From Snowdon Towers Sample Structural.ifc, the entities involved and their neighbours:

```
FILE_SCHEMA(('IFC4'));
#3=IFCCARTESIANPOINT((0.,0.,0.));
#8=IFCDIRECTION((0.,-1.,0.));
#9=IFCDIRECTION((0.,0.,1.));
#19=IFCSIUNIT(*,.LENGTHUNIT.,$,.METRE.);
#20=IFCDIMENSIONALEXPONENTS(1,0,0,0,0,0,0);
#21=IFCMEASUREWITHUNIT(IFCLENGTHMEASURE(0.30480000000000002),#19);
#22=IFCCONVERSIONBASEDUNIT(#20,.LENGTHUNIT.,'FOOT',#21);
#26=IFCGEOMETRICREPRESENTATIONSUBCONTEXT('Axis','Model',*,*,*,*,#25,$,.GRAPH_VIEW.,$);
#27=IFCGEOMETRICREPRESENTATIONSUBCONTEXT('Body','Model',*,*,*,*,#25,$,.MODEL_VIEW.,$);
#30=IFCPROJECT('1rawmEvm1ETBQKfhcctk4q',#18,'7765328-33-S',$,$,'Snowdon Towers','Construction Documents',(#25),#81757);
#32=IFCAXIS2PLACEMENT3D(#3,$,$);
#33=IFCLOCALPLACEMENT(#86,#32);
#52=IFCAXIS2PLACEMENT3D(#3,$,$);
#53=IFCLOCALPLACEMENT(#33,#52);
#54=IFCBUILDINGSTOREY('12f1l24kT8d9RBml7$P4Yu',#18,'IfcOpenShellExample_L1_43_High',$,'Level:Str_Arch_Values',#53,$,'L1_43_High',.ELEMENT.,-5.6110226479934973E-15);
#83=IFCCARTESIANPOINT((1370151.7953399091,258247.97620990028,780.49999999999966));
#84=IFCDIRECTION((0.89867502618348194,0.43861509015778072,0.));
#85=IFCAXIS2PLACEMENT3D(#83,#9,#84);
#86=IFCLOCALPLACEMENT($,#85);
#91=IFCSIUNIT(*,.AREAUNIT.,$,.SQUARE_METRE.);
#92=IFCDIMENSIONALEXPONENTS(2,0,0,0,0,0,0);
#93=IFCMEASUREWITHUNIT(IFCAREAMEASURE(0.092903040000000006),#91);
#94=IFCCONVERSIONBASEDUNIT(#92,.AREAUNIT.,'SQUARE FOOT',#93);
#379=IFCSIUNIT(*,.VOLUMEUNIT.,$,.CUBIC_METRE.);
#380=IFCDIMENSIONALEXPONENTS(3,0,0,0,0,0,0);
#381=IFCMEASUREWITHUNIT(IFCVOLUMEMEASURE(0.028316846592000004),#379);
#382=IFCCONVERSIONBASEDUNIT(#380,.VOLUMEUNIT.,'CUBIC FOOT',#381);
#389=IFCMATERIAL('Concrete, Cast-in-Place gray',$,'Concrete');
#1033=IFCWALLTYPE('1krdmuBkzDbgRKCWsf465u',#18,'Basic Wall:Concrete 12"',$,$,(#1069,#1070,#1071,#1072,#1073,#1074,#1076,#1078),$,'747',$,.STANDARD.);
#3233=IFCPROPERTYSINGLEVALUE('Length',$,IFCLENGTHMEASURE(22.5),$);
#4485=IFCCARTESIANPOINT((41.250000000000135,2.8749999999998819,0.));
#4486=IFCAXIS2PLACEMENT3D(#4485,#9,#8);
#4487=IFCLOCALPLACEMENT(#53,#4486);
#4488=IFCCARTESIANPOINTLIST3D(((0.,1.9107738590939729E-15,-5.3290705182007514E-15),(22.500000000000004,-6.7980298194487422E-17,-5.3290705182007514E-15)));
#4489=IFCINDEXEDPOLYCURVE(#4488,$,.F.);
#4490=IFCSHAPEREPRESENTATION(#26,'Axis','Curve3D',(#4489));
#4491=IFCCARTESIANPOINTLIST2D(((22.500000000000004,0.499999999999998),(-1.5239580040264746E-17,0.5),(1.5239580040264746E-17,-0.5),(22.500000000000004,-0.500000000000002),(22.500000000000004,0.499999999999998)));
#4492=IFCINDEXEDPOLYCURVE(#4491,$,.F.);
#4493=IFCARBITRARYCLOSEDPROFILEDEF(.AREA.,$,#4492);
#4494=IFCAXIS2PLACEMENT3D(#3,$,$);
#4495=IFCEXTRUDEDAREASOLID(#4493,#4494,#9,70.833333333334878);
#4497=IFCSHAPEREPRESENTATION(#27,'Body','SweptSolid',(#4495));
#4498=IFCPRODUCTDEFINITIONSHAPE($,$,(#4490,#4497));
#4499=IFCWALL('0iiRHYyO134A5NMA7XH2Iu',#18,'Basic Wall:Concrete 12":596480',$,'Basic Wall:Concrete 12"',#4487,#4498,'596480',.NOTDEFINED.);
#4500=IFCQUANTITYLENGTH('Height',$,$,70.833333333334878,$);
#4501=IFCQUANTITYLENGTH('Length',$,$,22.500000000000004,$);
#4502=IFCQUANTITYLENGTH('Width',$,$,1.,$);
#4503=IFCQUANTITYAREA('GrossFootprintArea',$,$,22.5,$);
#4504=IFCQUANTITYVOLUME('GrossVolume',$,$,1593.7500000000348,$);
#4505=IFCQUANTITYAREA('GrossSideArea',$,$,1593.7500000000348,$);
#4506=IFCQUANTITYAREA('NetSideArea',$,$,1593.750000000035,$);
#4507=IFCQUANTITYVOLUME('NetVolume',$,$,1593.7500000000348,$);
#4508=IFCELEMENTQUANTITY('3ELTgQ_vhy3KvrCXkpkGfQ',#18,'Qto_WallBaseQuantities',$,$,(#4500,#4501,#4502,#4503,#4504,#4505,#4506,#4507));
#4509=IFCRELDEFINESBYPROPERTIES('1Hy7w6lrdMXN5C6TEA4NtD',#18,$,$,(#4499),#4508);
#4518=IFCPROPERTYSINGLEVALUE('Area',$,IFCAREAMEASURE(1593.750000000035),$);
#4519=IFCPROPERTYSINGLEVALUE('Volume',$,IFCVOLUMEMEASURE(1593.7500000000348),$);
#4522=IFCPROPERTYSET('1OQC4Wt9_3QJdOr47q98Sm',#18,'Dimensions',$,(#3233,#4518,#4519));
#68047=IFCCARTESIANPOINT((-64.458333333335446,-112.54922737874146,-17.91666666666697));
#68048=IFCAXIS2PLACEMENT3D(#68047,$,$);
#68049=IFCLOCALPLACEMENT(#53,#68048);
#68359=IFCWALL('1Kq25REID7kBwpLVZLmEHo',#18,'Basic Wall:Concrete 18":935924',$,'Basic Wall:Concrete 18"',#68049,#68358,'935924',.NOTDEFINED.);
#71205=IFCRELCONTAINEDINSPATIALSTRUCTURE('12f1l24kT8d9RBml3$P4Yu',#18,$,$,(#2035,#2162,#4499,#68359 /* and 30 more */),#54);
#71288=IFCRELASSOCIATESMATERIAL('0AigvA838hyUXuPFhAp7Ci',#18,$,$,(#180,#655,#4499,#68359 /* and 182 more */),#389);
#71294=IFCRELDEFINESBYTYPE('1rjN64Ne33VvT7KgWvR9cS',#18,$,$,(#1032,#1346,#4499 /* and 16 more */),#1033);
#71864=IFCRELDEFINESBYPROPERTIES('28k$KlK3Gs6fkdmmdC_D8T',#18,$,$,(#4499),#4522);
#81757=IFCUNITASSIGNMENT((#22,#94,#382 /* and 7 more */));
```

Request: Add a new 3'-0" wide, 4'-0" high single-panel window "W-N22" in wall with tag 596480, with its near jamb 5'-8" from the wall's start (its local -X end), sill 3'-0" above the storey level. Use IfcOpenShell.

```python
import numpy as np
import ifcopenshell
import ifcopenshell.api.feature
import ifcopenshell.api.geometry
import ifcopenshell.api.pset
import ifcopenshell.api.root
import ifcopenshell.api.spatial
import ifcopenshell.geom
import ifcopenshell.util.element
import ifcopenshell.util.placement
import ifcopenshell.util.representation
import ifcopenshell.util.shape
import ifcopenshell.util.unit

model = ifcopenshell.open("Snowdon Towers Sample Structural.ifc")
unit_scale = ifcopenshell.util.unit.calculate_unit_scale(model)
area_scale = ifcopenshell.util.unit.calculate_unit_scale(model, "AREAUNIT")
volume_scale = ifcopenshell.util.unit.calculate_unit_scale(model, "VOLUMEUNIT")
settings = ifcopenshell.geom.settings()


def volume(element):
    """Net volume in cubic metres, openings subtracted."""
    shape = ifcopenshell.geom.create_shape(settings, element)
    return ifcopenshell.util.shape.get_volume(shape.geometry)


wall = model.by_guid("0iiRHYyO134A5NMA7XH2Iu")
storey = ifcopenshell.util.element.get_container(wall, ifc_class="IfcBuildingStorey")
context = ifcopenshell.util.representation.get_context(model, "Model", "Body", "MODEL_VIEW")
before = volume(wall)

width, height, from_end, sill = 0.9144, 1.2192, 1.7272, 0.9144  # metres

# The wall runs along its own X axis, and the end named is its -X end.
wall_shape = ifcopenshell.geom.create_shape(settings, wall)
x, y, z = ifcopenshell.util.shape.get_vertices(wall_shape.geometry).T
start = x.min() + from_end
face, thickness = float(y.min()), float(y.max() - y.min())
wall_matrix = ifcopenshell.util.placement.get_local_placement(wall.ObjectPlacement)
level = ifcopenshell.util.placement.get_local_placement(storey.ObjectPlacement)[2, 3]


def in_wall(x, y):
    """Placement at x, y metres in the wall's axes, at sill height."""
    matrix = wall_matrix.copy()
    matrix[:, 3] = wall_matrix @ np.array([x / unit_scale, y / unit_scale, 0.0, 1.0])
    matrix[2, 3] = level + sill / unit_scale
    return matrix


# Opening: a box that overshoots both wall faces by 50 mm.
opening = ifcopenshell.api.root.create_entity(model, ifc_class="IfcOpeningElement", predefined_type="OPENING")
box = ifcopenshell.api.geometry.add_wall_representation(
    model, context=context, length=width, height=height, thickness=thickness + 0.1
)
ifcopenshell.api.geometry.assign_representation(model, product=opening, representation=box)
ifcopenshell.api.geometry.edit_object_placement(model, product=opening, matrix=in_wall(start, face - 0.05), is_si=False)
ifcopenshell.api.feature.add_feature(model, feature=opening, element=wall)

window = ifcopenshell.api.root.create_entity(model, ifc_class="IfcWindow", name="W-N22", predefined_type="WINDOW")
window.OverallWidth, window.OverallHeight = width / unit_scale, height / unit_scale
window.PartitioningType = "SINGLE_PANEL"
body = ifcopenshell.api.geometry.add_window_representation(
    model,
    context=context,
    overall_width=window.OverallWidth,
    overall_height=window.OverallHeight,
    partition_type="SINGLE_PANEL",
)
ifcopenshell.api.geometry.assign_representation(model, product=window, representation=body)
ifcopenshell.api.spatial.assign_container(model, products=[window], relating_structure=storey)
ifcopenshell.api.feature.add_filling(model, opening=opening, element=window)

# Centre the window in the wall's thickness.
ifcopenshell.api.geometry.edit_object_placement(model, product=window, matrix=in_wall(start, face), is_si=False)
window_shape = ifcopenshell.geom.create_shape(settings, window)
depth = ifcopenshell.util.shape.get_vertices(window_shape.geometry)[:, 1]
offset = face + thickness / 2 - (depth.min() + depth.max()) / 2
ifcopenshell.api.geometry.edit_object_placement(model, product=window, matrix=in_wall(start, offset), is_si=False)

after = volume(wall)

# Update the wall's stored quantities.
qto = model.by_id(ifcopenshell.util.element.get_pset(wall, "Qto_WallBaseQuantities", should_inherit=False)["id"])
ifcopenshell.api.pset.edit_qto(model, qto=qto, properties={
    "NetSideArea": after / thickness / area_scale,
    "NetVolume": after / volume_scale,
})
pset = model.by_id(ifcopenshell.util.element.get_pset(wall, "Dimensions", should_inherit=False)["id"])
ifcopenshell.api.pset.edit_pset(model, pset=pset, properties={
    "Area": model.create_entity("IfcAreaMeasure", after / thickness / area_scale),
    "Volume": model.create_entity("IfcVolumeMeasure", after / volume_scale),
})

print(f"wall volume {before:.3f} -> {after:.3f} m3")

model.write("Snowdon Towers Sample Structural_rev.ifc")
```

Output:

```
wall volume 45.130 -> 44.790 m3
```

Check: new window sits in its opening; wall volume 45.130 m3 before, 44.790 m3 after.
